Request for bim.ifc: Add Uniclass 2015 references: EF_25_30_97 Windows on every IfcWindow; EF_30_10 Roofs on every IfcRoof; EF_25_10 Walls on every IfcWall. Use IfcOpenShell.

First a look at what the model holds.

```python
import ifcopenshell

model = ifcopenshell.open("bim.ifc")
print(model.schema)
print("classifications:", [c.Name for c in model.by_type("IfcClassification")])
for ifc_class in ("IfcDoor", "IfcRoof", "IfcStair", "IfcWall", "IfcWindow"):
    print(ifc_class, len(model.by_type(ifc_class)))
```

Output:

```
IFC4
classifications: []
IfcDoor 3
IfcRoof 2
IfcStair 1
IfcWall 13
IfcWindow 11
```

```python
import ifcopenshell
import ifcopenshell.api.classification

model = ifcopenshell.open("bim.ifc")

system = ifcopenshell.api.classification.add_classification(model, classification="Uniclass 2015")

codes = {
    "IfcWindow": ("EF_25_30_97", "Windows"),
    "IfcRoof": ("EF_30_10", "Roofs"),
    "IfcWall": ("EF_25_10", "Walls"),
}
for ifc_class, (code, name) in codes.items():
    products = model.by_type(ifc_class)
    ifcopenshell.api.classification.add_reference(
        model, products=products, classification=system, identification=code, name=name
    )
    print(code, len(products))

model.write("bim_updated.ifc")
```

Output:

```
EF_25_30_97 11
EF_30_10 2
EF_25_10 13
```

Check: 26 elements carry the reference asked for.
